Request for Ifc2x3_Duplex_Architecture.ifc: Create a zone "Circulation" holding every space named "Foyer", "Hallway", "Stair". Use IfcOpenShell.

First a look at what the model holds.

```python
import ifcopenshell

model = ifcopenshell.open("Ifc2x3_Duplex_Architecture.ifc")
print(model.schema)
seen = {}
for space in model.by_type("IfcSpace"):
    seen[space.LongName] = seen.get(space.LongName, 0) + 1
for name, count in sorted(seen.items(), key=str):
    print(count, "x", name)
print("zones:", [z.Name for z in model.by_type("IfcZone")][:20])
```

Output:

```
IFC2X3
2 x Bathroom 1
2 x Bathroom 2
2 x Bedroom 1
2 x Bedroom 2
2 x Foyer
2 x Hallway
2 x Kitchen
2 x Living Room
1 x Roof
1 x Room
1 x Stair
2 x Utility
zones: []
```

```python
import ifcopenshell
import ifcopenshell.api.group
import ifcopenshell.api.root

model = ifcopenshell.open("Ifc2x3_Duplex_Architecture.ifc")

names = {"Foyer", "Hallway", "Stair"}
spaces = [s for s in model.by_type("IfcSpace") if s.LongName in names]

zone = ifcopenshell.api.root.create_entity(model, ifc_class="IfcZone", name="Circulation")
ifcopenshell.api.group.assign_group(model, products=spaces, group=zone)
print(len(spaces), "spaces in", zone.Name)

model.write("Ifc2x3_Duplex_Architecture_edited.ifc")
```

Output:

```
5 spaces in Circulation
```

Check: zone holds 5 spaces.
